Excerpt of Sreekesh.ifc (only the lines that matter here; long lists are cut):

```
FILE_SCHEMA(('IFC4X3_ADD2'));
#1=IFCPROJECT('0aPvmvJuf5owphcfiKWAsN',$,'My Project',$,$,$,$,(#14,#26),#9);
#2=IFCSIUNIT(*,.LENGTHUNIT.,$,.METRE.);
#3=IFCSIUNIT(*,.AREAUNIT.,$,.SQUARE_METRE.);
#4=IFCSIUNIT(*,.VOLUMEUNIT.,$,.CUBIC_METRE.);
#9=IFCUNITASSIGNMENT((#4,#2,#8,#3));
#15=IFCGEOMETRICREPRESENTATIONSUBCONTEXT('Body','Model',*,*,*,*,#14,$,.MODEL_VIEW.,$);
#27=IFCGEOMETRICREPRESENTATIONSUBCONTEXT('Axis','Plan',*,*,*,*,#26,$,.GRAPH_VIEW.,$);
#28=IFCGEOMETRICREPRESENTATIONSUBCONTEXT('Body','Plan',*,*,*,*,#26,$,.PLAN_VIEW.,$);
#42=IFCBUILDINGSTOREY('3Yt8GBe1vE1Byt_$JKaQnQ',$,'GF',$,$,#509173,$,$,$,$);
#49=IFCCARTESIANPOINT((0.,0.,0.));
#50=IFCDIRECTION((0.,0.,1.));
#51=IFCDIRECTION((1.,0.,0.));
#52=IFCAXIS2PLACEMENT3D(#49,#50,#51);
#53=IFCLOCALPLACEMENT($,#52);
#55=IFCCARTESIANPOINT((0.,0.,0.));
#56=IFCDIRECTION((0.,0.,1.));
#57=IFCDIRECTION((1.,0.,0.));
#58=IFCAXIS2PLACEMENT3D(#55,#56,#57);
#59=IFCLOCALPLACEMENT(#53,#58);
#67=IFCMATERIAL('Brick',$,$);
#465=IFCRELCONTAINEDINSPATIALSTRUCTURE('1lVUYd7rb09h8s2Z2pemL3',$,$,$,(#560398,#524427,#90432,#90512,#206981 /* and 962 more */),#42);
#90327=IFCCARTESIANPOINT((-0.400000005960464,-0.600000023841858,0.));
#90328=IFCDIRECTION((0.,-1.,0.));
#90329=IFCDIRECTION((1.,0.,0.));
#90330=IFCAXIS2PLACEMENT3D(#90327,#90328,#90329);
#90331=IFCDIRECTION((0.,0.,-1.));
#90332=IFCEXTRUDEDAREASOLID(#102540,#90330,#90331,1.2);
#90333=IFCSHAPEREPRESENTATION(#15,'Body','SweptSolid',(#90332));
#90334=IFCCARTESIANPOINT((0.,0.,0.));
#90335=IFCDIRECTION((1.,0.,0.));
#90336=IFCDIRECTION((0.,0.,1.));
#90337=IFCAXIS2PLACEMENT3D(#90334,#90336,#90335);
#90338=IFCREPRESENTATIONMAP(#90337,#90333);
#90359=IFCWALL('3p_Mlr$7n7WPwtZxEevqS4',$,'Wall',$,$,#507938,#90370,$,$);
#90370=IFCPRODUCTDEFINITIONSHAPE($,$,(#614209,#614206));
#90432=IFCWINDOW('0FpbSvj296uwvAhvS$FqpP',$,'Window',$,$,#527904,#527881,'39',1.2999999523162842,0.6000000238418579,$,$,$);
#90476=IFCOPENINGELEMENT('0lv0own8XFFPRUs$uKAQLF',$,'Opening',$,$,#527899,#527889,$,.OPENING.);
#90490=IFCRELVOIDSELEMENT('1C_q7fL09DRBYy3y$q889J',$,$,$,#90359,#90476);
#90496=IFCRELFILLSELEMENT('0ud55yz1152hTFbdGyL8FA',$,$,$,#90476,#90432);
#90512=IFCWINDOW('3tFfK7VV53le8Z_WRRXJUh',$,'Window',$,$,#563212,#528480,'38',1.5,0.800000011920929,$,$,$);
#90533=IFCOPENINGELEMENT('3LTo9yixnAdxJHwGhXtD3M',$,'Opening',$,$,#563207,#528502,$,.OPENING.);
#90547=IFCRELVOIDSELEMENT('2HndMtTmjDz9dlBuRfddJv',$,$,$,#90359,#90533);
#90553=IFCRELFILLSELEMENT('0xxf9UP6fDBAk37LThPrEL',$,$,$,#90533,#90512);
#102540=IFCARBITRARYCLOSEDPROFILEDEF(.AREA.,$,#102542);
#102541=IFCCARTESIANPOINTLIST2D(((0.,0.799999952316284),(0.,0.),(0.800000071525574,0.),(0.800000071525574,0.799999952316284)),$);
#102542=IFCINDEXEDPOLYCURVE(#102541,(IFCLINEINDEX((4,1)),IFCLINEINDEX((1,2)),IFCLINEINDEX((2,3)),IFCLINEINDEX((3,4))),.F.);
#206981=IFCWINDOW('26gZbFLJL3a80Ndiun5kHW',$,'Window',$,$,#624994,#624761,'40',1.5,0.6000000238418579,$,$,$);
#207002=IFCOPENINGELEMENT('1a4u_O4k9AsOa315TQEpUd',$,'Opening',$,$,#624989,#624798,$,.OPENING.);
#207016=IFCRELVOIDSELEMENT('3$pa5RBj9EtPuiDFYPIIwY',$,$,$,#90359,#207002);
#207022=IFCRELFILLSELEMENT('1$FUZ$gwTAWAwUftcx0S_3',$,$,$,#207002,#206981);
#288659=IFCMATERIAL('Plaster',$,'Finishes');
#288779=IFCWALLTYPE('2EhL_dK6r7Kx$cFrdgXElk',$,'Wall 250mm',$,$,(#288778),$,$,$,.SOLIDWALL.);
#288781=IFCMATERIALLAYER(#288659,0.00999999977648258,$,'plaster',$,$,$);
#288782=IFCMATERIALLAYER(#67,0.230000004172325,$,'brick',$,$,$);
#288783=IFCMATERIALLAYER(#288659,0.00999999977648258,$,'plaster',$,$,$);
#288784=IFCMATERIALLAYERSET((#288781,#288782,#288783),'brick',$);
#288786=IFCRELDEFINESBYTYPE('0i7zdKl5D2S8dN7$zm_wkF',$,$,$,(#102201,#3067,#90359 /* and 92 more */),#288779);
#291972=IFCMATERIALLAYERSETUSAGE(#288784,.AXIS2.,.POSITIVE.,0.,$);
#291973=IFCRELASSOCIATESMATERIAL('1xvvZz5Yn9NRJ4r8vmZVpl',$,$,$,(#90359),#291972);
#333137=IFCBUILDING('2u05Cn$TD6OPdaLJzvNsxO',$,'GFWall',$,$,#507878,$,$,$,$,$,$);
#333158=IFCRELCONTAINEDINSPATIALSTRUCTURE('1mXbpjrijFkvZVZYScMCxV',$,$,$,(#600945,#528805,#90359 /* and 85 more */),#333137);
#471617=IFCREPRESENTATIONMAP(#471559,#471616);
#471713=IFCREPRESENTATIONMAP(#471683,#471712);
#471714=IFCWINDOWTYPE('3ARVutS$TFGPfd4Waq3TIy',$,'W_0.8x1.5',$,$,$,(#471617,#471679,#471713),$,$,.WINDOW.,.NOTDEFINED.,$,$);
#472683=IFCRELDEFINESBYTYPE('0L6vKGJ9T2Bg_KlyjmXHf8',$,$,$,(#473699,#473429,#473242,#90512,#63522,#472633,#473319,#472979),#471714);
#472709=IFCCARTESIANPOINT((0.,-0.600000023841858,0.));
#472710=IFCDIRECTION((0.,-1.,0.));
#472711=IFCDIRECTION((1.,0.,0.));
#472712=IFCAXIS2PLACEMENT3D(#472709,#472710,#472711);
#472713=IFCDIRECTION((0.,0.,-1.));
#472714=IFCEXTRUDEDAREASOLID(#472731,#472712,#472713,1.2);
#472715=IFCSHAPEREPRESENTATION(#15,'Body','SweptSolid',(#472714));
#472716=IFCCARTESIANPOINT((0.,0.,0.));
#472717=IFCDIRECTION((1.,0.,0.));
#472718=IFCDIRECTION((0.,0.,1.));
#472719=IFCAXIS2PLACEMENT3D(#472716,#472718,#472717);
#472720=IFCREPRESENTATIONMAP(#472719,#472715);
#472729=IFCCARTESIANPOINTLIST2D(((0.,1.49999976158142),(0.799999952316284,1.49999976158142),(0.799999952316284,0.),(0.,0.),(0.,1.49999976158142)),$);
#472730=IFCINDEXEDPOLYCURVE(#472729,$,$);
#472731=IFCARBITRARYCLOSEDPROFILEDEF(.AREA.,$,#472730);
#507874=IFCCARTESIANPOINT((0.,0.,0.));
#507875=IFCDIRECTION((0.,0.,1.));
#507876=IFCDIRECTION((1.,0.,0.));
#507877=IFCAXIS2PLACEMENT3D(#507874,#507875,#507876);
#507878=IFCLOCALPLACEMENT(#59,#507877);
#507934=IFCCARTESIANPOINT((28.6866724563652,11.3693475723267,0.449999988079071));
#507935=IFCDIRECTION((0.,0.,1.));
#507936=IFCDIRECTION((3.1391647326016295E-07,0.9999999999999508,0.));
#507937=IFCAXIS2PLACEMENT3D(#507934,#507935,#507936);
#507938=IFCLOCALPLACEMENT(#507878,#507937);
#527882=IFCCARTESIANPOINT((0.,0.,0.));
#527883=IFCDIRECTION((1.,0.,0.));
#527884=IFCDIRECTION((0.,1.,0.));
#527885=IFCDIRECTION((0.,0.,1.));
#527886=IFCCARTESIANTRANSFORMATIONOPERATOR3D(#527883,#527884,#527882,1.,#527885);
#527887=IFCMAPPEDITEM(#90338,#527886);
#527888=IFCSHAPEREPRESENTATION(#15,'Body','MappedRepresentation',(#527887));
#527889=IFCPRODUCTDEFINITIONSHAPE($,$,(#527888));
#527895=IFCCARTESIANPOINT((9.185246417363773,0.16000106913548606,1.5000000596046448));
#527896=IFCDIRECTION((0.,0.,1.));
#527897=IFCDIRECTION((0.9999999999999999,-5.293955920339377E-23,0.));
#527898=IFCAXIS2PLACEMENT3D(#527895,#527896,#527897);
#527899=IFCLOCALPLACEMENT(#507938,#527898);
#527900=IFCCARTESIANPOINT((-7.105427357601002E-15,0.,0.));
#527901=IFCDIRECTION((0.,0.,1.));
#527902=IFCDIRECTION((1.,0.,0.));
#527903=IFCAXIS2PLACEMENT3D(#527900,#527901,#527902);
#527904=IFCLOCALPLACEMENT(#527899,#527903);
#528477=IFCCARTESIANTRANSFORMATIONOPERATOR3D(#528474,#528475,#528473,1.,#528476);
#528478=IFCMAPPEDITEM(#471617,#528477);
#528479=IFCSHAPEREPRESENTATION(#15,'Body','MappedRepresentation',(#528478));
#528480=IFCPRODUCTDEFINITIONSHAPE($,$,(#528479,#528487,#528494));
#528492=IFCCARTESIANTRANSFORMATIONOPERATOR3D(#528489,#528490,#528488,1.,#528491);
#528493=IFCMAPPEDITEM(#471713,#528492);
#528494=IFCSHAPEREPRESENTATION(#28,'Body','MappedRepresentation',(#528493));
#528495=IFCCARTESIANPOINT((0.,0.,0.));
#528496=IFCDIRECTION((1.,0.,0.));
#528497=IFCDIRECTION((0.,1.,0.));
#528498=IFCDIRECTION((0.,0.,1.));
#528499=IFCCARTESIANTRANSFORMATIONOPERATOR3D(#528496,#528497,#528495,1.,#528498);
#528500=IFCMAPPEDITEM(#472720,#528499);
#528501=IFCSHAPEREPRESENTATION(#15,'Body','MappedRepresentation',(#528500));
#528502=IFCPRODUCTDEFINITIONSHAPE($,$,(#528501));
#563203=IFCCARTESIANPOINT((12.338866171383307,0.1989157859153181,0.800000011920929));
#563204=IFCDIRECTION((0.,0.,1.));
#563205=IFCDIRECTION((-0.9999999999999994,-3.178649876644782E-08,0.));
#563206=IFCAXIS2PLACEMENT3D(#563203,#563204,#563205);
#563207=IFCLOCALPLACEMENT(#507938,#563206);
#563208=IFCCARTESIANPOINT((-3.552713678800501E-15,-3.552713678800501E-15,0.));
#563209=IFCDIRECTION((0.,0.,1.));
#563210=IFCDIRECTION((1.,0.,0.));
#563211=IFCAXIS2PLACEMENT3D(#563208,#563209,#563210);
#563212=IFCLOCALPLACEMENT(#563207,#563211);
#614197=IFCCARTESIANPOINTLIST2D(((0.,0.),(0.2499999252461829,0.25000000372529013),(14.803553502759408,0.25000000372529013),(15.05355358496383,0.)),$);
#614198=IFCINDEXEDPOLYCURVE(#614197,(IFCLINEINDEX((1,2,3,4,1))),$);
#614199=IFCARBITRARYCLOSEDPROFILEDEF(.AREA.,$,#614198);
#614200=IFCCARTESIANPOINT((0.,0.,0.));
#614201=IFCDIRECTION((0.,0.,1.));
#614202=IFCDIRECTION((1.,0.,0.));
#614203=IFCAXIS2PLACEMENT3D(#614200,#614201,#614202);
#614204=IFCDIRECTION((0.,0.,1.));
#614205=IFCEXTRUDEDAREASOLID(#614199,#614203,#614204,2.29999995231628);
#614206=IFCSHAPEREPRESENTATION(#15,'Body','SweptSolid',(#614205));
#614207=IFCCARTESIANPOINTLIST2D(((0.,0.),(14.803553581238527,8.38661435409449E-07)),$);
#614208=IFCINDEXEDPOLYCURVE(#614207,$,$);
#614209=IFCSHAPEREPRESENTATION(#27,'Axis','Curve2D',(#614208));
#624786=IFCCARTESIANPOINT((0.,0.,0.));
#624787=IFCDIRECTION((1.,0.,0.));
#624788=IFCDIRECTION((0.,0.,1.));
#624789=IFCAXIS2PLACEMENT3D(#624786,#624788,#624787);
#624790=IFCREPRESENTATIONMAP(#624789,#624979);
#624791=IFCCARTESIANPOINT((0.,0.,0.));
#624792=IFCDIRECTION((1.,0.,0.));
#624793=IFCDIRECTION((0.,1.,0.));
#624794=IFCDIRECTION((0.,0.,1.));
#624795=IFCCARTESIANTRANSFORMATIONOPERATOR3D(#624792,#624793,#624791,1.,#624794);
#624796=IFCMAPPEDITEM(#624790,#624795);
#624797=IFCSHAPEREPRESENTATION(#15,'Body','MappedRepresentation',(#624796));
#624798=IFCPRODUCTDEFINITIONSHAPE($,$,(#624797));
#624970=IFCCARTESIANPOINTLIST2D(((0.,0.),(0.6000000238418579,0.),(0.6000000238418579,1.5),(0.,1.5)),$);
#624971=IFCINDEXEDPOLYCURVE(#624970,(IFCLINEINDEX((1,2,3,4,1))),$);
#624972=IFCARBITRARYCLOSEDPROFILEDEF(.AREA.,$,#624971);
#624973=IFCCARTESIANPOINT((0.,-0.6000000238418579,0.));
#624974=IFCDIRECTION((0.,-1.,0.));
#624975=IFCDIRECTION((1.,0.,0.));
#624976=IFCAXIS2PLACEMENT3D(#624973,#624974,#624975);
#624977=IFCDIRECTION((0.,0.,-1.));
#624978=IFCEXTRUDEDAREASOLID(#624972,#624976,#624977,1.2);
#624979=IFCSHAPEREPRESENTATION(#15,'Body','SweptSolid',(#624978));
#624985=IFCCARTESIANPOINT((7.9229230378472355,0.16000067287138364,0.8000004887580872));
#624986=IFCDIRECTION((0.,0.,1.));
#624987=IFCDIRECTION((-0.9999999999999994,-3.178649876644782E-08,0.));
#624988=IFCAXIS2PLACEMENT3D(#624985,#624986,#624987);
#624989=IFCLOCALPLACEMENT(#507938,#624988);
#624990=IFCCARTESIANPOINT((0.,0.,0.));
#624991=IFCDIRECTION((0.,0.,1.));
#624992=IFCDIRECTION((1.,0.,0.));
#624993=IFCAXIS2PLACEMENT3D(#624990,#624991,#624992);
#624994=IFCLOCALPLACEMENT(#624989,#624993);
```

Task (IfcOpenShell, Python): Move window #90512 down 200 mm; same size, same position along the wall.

```python
import numpy as np
import ifcopenshell
import ifcopenshell.api.geometry
import ifcopenshell.util.placement
import ifcopenshell.util.unit

model = ifcopenshell.open("Sreekesh.ifc")
unit_scale = ifcopenshell.util.unit.calculate_unit_scale(model)

window = model.by_id(90512)
opening = window.FillsVoids[0].RelatingOpeningElement
dz = -0.2 / unit_scale

shift = np.array([0.0, 0.0, dz])
# The window is placed relative to its opening, so it follows when the opening moves.
matrix = ifcopenshell.util.placement.get_local_placement(opening.ObjectPlacement)
matrix[:3, 3] += shift
ifcopenshell.api.geometry.edit_object_placement(
    model, product=opening, matrix=matrix, is_si=False, should_transform_children=True
)

print(f"moved by {dz * unit_scale:+.3f} m")

model.write("Sreekesh_updated.ifc")
```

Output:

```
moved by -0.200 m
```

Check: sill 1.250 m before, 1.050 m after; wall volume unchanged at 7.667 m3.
